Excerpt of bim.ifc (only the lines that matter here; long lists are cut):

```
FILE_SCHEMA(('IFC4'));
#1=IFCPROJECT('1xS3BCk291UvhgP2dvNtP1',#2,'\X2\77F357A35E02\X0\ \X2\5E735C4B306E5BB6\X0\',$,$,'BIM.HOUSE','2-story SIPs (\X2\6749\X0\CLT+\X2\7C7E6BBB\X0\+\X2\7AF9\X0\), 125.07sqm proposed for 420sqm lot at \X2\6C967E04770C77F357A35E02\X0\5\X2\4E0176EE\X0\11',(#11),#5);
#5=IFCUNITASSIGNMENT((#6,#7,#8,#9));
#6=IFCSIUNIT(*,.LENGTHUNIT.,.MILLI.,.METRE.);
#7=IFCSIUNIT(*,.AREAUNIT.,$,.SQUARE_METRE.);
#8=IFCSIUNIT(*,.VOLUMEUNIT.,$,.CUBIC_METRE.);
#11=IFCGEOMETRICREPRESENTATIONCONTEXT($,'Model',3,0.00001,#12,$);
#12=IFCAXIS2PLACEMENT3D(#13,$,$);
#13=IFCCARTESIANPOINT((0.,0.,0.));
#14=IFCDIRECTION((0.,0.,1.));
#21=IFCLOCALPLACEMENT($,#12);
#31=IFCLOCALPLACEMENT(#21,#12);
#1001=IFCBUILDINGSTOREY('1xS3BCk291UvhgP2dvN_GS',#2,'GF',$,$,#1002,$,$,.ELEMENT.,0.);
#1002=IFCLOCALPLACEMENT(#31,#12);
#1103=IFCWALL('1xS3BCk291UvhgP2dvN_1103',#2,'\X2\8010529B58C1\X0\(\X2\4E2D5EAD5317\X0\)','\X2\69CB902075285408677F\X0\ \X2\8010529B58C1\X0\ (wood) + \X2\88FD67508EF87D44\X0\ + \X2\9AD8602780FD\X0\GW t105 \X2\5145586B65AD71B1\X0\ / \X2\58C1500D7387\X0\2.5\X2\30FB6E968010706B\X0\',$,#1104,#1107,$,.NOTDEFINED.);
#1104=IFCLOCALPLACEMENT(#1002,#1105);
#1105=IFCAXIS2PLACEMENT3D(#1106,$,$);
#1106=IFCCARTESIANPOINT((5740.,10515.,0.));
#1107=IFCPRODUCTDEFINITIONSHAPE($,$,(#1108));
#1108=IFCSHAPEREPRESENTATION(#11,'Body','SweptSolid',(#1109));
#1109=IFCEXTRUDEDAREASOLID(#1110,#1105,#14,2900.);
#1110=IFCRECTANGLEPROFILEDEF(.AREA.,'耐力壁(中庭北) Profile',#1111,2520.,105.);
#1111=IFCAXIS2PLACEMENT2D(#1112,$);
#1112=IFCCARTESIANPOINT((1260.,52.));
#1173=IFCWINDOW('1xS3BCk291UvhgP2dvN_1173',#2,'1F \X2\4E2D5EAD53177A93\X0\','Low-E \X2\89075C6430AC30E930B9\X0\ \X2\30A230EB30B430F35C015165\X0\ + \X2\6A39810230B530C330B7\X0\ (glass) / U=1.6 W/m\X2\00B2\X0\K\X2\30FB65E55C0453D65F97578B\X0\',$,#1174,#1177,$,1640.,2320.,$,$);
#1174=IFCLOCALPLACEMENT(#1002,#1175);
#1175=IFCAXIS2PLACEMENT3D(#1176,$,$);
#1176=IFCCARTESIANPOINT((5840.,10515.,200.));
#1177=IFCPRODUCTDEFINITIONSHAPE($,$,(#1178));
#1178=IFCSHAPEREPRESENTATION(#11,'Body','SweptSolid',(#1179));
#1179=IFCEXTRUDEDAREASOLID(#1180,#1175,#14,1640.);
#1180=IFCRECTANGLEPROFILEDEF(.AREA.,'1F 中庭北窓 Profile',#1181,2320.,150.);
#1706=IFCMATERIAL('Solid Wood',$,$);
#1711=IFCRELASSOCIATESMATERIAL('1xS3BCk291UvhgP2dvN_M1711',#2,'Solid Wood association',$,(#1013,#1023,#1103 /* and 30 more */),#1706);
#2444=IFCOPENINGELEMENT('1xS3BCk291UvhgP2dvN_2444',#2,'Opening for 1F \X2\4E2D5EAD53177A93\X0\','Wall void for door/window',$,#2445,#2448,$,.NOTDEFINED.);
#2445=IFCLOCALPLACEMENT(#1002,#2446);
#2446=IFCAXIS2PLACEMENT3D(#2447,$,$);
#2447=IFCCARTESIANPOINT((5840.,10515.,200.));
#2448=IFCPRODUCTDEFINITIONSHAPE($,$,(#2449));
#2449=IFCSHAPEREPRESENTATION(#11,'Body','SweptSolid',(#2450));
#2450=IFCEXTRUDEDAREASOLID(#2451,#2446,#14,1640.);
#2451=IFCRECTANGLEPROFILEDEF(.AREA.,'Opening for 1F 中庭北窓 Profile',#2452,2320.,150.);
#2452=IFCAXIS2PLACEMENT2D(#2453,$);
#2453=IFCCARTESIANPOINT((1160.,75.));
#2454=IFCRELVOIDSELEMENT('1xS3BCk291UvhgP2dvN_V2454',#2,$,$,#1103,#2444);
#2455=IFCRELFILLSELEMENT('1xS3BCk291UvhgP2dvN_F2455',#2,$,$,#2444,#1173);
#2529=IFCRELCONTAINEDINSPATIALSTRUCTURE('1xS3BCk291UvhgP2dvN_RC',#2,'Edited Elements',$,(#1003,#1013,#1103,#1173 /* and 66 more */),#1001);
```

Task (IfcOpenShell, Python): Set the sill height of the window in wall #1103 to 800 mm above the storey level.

```python
import numpy as np
import ifcopenshell
import ifcopenshell.api.geometry
import ifcopenshell.geom
import ifcopenshell.util.element
import ifcopenshell.util.placement
import ifcopenshell.util.shape
import ifcopenshell.util.unit

model = ifcopenshell.open("bim.ifc")
unit_scale = ifcopenshell.util.unit.calculate_unit_scale(model)

window = model.by_guid("1xS3BCk291UvhgP2dvN_1173")
opening = window.FillsVoids[0].RelatingOpeningElement
storey = ifcopenshell.util.element.get_container(window, ifc_class="IfcBuildingStorey")
level = ifcopenshell.util.placement.get_local_placement(storey.ObjectPlacement)[2, 3]

# The opening's origin need not be at the sill, so measure its lowest point.
shape = ifcopenshell.geom.create_shape(ifcopenshell.geom.settings(), opening)
bottom = ifcopenshell.util.shape.get_shape_bottom_elevation(shape, shape.geometry) / unit_scale
dz = level + 0.8 / unit_scale - bottom

shift = np.array([0.0, 0.0, dz])
# The window is not placed relative to its opening, so move both.
for product in (opening, window):
    matrix = ifcopenshell.util.placement.get_local_placement(product.ObjectPlacement)
    matrix[:3, 3] += shift
    ifcopenshell.api.geometry.edit_object_placement(model, product=product, matrix=matrix, is_si=False)

print(f"moved by {dz * unit_scale:+.3f} m")

model.write("bim_rev.ifc")
```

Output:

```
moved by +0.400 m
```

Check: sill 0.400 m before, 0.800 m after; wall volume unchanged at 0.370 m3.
